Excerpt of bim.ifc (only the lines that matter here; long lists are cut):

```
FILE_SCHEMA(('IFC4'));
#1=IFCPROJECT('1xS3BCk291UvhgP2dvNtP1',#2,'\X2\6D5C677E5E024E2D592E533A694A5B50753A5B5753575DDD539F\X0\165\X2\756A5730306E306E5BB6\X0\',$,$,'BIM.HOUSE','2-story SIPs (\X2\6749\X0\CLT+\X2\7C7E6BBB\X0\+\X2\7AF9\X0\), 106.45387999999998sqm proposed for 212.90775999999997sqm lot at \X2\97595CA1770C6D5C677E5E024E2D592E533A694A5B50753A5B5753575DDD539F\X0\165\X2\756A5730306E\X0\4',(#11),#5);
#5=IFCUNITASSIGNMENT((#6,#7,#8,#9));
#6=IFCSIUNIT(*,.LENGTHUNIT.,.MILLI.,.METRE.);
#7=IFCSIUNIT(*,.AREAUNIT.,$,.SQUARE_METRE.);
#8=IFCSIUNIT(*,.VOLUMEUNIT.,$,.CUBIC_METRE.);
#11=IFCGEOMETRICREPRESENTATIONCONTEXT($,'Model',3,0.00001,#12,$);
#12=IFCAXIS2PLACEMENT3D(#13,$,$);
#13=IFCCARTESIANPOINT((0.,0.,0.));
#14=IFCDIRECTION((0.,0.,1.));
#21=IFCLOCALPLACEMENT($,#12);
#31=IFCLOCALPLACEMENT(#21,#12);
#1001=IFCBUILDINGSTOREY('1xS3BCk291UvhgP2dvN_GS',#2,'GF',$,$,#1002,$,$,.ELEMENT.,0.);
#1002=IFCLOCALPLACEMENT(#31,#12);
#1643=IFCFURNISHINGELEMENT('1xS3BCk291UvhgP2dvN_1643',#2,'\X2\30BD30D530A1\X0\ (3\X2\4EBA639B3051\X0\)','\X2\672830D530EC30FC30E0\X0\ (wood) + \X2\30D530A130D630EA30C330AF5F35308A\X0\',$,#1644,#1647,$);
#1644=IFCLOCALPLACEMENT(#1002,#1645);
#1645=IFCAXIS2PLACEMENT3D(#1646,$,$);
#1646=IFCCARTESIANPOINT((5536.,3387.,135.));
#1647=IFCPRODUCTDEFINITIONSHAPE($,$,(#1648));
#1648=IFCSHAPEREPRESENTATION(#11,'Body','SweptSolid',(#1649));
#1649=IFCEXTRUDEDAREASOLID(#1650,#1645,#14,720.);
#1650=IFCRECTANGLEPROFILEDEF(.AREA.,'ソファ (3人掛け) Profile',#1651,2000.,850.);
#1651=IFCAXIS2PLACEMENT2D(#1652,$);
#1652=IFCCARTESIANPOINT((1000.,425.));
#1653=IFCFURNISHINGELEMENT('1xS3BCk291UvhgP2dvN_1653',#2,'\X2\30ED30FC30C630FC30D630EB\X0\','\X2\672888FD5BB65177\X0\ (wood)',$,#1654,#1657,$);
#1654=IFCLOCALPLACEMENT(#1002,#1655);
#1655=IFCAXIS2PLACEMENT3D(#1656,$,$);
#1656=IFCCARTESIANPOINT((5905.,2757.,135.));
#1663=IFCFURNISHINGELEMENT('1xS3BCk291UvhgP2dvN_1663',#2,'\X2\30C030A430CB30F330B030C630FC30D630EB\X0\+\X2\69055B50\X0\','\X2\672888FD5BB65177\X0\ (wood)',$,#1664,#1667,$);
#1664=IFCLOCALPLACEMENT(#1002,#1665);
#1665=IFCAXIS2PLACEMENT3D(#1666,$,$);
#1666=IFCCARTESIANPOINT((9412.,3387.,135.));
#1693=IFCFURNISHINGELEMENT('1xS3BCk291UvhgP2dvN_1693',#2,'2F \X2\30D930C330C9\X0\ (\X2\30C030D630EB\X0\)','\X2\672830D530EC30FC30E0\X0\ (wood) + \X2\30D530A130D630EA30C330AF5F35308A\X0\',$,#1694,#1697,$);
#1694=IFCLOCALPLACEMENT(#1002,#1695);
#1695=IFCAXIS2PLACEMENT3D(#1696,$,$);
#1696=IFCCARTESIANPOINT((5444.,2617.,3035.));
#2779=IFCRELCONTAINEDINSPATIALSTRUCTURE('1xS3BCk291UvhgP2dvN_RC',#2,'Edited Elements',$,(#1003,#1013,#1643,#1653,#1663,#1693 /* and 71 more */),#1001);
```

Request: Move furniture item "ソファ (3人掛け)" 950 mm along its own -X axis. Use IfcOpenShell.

```python
import ifcopenshell
import ifcopenshell.api.geometry
import ifcopenshell.util.placement

model = ifcopenshell.open("bim.ifc")

item = model.by_guid("1xS3BCk291UvhgP2dvN_1643")
matrix = ifcopenshell.util.placement.get_local_placement(item.ObjectPlacement)
matrix[:3, 3] -= matrix[:3, 0] * 950.0
ifcopenshell.api.geometry.edit_object_placement(model, product=item, matrix=matrix, is_si=False)

print(ifcopenshell.util.placement.get_local_placement(item.ObjectPlacement).round(3) + 0.0)

model.write("bim_edited.ifc")
```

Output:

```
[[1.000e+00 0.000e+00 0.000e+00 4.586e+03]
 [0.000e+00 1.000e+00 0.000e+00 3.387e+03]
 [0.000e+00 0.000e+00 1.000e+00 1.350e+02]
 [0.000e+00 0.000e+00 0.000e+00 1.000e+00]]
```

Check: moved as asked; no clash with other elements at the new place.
